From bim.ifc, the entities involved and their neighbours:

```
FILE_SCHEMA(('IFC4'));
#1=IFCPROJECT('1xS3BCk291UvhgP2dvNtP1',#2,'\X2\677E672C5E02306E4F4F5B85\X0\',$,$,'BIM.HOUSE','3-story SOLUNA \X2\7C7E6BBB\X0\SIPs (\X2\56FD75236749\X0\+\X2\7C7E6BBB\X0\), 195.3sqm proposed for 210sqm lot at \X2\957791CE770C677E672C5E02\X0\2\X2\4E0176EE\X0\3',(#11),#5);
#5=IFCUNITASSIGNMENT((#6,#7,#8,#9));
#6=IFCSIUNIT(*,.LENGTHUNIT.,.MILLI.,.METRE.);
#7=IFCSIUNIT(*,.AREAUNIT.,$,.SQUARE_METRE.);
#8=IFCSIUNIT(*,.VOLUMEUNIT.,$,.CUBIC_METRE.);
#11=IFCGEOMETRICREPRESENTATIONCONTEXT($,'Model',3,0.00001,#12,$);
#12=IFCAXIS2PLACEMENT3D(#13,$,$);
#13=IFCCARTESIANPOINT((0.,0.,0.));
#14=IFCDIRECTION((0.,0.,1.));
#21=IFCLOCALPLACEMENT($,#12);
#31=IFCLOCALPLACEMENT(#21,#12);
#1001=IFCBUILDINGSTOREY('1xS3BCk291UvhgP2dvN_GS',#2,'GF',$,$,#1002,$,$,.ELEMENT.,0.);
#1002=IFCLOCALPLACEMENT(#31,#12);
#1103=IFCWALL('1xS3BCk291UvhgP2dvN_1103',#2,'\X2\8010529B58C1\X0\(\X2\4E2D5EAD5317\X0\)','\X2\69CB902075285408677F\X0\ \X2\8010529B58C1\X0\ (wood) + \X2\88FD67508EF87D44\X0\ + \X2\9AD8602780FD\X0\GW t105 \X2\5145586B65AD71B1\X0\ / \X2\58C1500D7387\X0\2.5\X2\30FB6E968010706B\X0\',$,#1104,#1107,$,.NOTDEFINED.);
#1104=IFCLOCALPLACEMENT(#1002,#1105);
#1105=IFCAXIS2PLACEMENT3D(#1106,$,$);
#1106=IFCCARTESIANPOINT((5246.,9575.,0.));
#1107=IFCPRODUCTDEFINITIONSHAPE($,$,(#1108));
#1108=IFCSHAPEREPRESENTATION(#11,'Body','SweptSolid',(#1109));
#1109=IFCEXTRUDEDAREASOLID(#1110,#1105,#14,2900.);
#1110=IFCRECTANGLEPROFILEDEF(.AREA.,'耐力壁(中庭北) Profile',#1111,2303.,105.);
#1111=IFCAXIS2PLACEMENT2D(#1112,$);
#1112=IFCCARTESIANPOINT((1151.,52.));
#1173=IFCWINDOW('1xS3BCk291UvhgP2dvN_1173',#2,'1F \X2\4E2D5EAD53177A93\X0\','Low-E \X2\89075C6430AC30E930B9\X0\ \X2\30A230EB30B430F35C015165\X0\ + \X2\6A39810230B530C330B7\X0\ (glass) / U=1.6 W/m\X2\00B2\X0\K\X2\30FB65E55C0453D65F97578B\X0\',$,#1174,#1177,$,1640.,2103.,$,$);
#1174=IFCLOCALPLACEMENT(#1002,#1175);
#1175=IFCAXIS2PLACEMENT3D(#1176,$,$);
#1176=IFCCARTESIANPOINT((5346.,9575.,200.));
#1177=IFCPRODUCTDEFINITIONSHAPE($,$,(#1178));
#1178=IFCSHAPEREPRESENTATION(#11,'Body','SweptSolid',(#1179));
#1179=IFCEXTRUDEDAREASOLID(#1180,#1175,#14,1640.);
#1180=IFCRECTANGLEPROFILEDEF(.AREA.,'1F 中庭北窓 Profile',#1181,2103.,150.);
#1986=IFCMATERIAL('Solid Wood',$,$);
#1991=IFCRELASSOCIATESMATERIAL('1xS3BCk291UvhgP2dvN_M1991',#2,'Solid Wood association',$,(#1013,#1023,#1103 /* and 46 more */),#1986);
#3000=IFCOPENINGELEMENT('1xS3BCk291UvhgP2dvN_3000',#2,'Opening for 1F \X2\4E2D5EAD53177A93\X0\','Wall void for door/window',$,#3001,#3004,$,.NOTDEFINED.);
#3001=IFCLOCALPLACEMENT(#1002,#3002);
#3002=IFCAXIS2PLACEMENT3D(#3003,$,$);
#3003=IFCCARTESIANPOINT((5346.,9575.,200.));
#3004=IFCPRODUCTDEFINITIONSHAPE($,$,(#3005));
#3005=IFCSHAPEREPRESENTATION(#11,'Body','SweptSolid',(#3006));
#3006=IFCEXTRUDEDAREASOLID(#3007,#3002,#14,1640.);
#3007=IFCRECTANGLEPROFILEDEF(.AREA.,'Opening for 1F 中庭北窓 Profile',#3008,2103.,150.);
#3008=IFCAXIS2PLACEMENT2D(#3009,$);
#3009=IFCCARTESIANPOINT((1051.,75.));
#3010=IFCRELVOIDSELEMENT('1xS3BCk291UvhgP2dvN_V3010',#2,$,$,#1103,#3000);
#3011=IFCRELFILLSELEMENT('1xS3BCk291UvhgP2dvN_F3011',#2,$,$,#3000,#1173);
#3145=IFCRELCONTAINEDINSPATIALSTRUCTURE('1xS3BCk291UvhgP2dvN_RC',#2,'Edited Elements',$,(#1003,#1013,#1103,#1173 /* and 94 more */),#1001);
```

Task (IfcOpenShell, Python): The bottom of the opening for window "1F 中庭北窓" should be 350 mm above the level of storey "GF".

```python
import numpy as np
import ifcopenshell
import ifcopenshell.api.geometry
import ifcopenshell.geom
import ifcopenshell.util.element
import ifcopenshell.util.placement
import ifcopenshell.util.shape
import ifcopenshell.util.unit

model = ifcopenshell.open("bim.ifc")
unit_scale = ifcopenshell.util.unit.calculate_unit_scale(model)

window = model.by_guid("1xS3BCk291UvhgP2dvN_1173")
opening = window.FillsVoids[0].RelatingOpeningElement
storey = ifcopenshell.util.element.get_container(window, ifc_class="IfcBuildingStorey")
level = ifcopenshell.util.placement.get_local_placement(storey.ObjectPlacement)[2, 3]

# The opening's origin need not be at the sill, so measure its lowest point.
shape = ifcopenshell.geom.create_shape(ifcopenshell.geom.settings(), opening)
bottom = ifcopenshell.util.shape.get_shape_bottom_elevation(shape, shape.geometry) / unit_scale
dz = level + 0.35 / unit_scale - bottom

shift = np.array([0.0, 0.0, dz])
# The window is not placed relative to its opening, so move both.
for product in (opening, window):
    matrix = ifcopenshell.util.placement.get_local_placement(product.ObjectPlacement)
    matrix[:3, 3] += shift
    ifcopenshell.api.geometry.edit_object_placement(model, product=product, matrix=matrix, is_si=False)

print(f"moved by {dz * unit_scale:+.3f} m")

model.write("bim-out.ifc")
```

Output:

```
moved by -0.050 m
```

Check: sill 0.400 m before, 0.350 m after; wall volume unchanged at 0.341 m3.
